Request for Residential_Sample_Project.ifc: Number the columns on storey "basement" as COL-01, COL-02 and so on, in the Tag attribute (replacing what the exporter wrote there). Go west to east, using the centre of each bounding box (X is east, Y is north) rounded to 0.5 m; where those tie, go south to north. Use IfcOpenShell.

First a look at what the model holds.

```python
import ifcopenshell
import ifcopenshell.util.element
import ifcopenshell.util.placement

model = ifcopenshell.open("Residential_Sample_Project.ifc")
print(model.schema)
storey = next(s for s in model.by_type("IfcBuildingStorey") if s.Name == "basement")
columns = [e for e in ifcopenshell.util.element.get_decomposition(storey) if e.is_a("IfcColumn")]
for e in sorted(columns, key=lambda e: e.id()):
    origin = ifcopenshell.util.placement.get_local_placement(e.ObjectPlacement)[:3, 3]
    print(e.id(), e.Tag, e.Name, origin.round(2) + 0.0, sep=" | ")
```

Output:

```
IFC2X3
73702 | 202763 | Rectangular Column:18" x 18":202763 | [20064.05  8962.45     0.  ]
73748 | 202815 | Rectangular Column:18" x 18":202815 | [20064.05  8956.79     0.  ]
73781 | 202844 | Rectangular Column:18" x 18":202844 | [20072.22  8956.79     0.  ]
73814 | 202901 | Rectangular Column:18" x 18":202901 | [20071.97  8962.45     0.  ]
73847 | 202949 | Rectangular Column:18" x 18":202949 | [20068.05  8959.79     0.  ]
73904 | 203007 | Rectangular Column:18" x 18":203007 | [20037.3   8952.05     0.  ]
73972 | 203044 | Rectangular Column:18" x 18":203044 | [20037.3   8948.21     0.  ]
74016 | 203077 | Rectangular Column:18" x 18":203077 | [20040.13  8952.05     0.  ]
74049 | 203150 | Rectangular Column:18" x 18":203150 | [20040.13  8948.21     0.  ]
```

```python
import ifcopenshell
import ifcopenshell.geom
import ifcopenshell.util.element
import ifcopenshell.util.shape

model = ifcopenshell.open("Residential_Sample_Project.ifc")
settings = ifcopenshell.geom.settings()
settings.set("use-world-coords", True)


def centre(element):
    shape = ifcopenshell.geom.create_shape(settings, element)
    return ifcopenshell.util.shape.get_bbox_centroid(shape.geometry)


storey = next(s for s in model.by_type("IfcBuildingStorey") if s.Name == "basement")
columns = [e for e in ifcopenshell.util.element.get_decomposition(storey) if e.is_a("IfcColumn")]

# Insertion points can sit at a corner or the storey origin, so sort by the geometry (in metres).
centres = {e: centre(e) for e in columns}
columns.sort(key=lambda e: (round(centres[e][0] / 0.5), centres[e][1]))

for i, e in enumerate(columns, start=1):
    number = f"COL-{i:02d}"
    e.Tag = number
    print(e.id(), number)

model.write("Residential_Sample_Project-out.ifc")
```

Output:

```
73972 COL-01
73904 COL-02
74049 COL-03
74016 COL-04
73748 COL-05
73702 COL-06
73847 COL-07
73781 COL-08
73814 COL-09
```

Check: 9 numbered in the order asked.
